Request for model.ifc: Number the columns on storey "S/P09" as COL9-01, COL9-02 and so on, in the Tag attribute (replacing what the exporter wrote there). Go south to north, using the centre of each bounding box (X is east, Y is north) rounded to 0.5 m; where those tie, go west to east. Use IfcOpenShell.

First a look at what the model holds.

```python
import ifcopenshell
import ifcopenshell.util.element
import ifcopenshell.util.placement

model = ifcopenshell.open("model.ifc")
print(model.schema)
storey = next(s for s in model.by_type("IfcBuildingStorey") if s.Name == "S/P09")
columns = [e for e in ifcopenshell.util.element.get_decomposition(storey) if e.is_a("IfcColumn")]
for e in sorted(columns, key=lambda e: e.id()):
    origin = ifcopenshell.util.placement.get_local_placement(e.ObjectPlacement)[:3, 3]
    print(e.id(), e.Tag, e.Name, origin.round(2) + 0.0, sep=" | ")
```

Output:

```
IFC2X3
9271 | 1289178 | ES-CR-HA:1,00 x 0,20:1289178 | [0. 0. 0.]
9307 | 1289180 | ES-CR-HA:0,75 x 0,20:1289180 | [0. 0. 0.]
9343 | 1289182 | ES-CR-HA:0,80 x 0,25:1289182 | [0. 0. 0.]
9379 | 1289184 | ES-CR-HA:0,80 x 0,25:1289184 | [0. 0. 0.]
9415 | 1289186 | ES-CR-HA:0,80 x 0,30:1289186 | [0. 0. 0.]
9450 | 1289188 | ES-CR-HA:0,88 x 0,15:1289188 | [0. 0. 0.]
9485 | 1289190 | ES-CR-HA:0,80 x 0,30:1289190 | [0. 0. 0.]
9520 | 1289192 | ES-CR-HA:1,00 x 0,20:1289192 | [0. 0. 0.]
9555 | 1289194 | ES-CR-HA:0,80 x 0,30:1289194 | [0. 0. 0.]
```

```python
import ifcopenshell
import ifcopenshell.geom
import ifcopenshell.util.element
import ifcopenshell.util.shape

model = ifcopenshell.open("model.ifc")
settings = ifcopenshell.geom.settings()
settings.set("use-world-coords", True)


def centre(element):
    shape = ifcopenshell.geom.create_shape(settings, element)
    return ifcopenshell.util.shape.get_bbox_centroid(shape.geometry)


storey = next(s for s in model.by_type("IfcBuildingStorey") if s.Name == "S/P09")
columns = [e for e in ifcopenshell.util.element.get_decomposition(storey) if e.is_a("IfcColumn")]

# Insertion points can sit at a corner or the storey origin, so sort by the geometry (in metres).
centres = {e: centre(e) for e in columns}
columns.sort(key=lambda e: (round(centres[e][1] / 0.5), centres[e][0]))

for i, e in enumerate(columns, start=1):
    number = f"COL9-{i:02d}"
    e.Tag = number
    print(e.id(), number)

model.write("model_updated.ifc")
```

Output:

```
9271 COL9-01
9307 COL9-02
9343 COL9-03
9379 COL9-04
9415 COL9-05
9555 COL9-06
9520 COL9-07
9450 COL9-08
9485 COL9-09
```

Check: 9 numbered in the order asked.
